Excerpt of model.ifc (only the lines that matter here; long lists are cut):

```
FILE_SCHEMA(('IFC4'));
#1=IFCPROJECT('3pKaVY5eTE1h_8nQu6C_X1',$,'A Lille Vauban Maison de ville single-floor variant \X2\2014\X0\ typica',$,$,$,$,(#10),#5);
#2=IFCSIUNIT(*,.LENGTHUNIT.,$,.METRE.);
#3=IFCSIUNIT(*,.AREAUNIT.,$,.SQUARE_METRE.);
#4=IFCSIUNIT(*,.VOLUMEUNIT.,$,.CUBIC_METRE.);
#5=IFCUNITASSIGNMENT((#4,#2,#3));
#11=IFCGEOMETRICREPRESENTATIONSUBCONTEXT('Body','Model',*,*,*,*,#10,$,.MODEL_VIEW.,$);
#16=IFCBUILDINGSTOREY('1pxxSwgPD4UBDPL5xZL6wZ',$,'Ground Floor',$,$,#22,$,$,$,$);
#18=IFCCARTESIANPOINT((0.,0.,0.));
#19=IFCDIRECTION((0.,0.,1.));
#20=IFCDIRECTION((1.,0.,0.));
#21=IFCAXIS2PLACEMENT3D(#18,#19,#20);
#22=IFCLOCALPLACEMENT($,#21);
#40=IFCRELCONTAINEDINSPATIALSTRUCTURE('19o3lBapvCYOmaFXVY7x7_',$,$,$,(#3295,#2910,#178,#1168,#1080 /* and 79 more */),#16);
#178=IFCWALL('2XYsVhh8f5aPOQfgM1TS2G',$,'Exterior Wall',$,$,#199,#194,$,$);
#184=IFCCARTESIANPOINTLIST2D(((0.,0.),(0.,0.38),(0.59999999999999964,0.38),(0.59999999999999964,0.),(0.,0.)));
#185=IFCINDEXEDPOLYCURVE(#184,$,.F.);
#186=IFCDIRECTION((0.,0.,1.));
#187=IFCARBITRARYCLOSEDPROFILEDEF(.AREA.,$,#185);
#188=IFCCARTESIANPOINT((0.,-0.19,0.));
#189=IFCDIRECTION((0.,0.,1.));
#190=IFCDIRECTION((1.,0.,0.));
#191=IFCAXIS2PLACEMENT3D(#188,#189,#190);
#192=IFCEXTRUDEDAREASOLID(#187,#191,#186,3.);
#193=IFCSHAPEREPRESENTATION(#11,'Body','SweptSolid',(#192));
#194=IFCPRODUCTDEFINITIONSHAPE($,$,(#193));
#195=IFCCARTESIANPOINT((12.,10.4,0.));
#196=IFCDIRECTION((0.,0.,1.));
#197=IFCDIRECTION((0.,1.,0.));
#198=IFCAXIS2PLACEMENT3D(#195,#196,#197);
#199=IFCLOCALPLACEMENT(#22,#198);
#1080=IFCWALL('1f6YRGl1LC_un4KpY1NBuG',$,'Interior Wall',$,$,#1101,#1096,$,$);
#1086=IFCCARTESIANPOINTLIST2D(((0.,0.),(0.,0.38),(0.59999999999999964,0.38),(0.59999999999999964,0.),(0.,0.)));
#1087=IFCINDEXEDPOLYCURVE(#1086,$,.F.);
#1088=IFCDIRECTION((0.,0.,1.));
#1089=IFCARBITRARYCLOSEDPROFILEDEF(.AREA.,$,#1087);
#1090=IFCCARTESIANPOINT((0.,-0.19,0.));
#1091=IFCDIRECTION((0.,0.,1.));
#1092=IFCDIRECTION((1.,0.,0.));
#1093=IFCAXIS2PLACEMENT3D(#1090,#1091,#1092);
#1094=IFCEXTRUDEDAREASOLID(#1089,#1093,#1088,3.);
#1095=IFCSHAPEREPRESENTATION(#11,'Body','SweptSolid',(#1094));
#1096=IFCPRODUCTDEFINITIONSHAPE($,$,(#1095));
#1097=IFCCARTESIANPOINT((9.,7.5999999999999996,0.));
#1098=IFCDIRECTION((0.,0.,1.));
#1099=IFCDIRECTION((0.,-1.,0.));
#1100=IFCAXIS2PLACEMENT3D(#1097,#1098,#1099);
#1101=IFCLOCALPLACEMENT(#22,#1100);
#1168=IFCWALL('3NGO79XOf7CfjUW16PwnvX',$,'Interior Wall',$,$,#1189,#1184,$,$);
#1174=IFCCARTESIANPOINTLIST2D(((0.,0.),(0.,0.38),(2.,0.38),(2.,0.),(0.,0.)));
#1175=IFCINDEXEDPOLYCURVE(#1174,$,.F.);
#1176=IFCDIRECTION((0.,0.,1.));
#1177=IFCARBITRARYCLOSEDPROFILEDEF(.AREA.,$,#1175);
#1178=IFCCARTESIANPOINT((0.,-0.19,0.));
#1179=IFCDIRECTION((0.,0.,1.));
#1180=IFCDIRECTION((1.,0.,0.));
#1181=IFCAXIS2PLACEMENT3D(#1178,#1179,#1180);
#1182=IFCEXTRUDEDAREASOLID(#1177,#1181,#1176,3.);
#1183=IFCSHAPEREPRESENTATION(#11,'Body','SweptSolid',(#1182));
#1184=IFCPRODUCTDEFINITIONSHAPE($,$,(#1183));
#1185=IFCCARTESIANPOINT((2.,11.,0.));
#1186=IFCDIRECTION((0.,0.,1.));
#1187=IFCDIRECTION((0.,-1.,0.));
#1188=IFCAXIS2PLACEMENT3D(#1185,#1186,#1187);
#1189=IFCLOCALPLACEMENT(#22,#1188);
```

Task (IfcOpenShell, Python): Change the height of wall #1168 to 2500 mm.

```python
import ifcopenshell
import ifcopenshell.geom
import ifcopenshell.util.representation
import ifcopenshell.util.shape
import ifcopenshell.util.unit

model = ifcopenshell.open("model.ifc")
unit_scale = ifcopenshell.util.unit.calculate_unit_scale(model)
settings = ifcopenshell.geom.settings()


def volume(element):
    """Net volume in cubic metres, openings subtracted."""
    shape = ifcopenshell.geom.create_shape(settings, element)
    return ifcopenshell.util.shape.get_volume(shape.geometry)


wall = model.by_id(1168)
before = volume(wall)

body = ifcopenshell.util.representation.get_representation(wall, "Model", "Body")
solid = body.Items[0]
old_height = solid.Depth
solid.Depth = 2.5 / unit_scale
after = volume(wall)

print(f"height {old_height:g} -> {solid.Depth:g}, volume {before:.3f} -> {after:.3f} m3")

model.write("model_rev.ifc")
```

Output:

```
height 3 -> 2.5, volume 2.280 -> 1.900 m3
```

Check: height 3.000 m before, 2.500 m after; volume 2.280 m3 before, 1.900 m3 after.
